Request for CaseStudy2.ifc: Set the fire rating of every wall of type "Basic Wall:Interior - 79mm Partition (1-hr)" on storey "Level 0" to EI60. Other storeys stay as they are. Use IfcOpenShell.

First a look at what the model holds.

```python
import ifcopenshell
import ifcopenshell.util.element

model = ifcopenshell.open("CaseStudy2.ifc")
print(model.schema)
storey = next(s for s in model.by_type("IfcBuildingStorey") if s.Name == "Level 0")
walls = [e for e in ifcopenshell.util.element.get_decomposition(storey) if e.is_a("IfcWall")]
seen = {}
for e in walls:
    element_type = ifcopenshell.util.element.get_type(e)
    key = (element_type.Name if element_type != e and element_type else None, ifcopenshell.util.element.get_pset(e, "Pset_WallCommon", "FireRating"))
    seen[key] = seen.get(key, 0) + 1
for (name, value), count in sorted(seen.items(), key=str):
    print(count, "x", name, "|", value)
```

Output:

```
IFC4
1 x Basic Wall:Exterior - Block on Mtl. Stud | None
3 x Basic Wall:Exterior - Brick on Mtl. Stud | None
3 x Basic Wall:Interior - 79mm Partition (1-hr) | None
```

```python
import ifcopenshell
import ifcopenshell.api.pset
import ifcopenshell.util.element

model = ifcopenshell.open("CaseStudy2.ifc")

storey = next(s for s in model.by_type("IfcBuildingStorey") if s.Name == "Level 0")
walls = [e for e in ifcopenshell.util.element.get_decomposition(storey) if e.is_a("IfcWall")]

count = 0
for e in walls:
    element_type = ifcopenshell.util.element.get_type(e)
    if element_type in (None, e) or element_type.Name != "Basic Wall:Interior - 79mm Partition (1-hr)":
        continue
    # add_pset returns the element's existing set when there is one.
    pset = ifcopenshell.api.pset.add_pset(model, product=e, name="Pset_WallCommon")
    ifcopenshell.api.pset.edit_pset(model, pset=pset, properties={"FireRating": "EI60"})
    count += 1

print(count, "walls updated")

model.write("CaseStudy2-out.ifc")
```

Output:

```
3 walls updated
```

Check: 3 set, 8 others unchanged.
